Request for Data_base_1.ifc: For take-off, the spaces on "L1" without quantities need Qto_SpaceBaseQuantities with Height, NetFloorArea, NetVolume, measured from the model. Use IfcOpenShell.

First a look at what the model holds.

```python
import ifcopenshell
import ifcopenshell.util.element
import ifcopenshell.util.unit

model = ifcopenshell.open("Data_base_1.ifc")
print(model.schema)
for unit_type in ("LENGTHUNIT", "AREAUNIT", "VOLUMEUNIT"):
    print(unit_type, ifcopenshell.util.unit.calculate_unit_scale(model, unit_type))
storey = next(s for s in model.by_type("IfcBuildingStorey") if s.Name == "L1")
spaces = [e for e in ifcopenshell.util.element.get_decomposition(storey) if e.is_a("IfcSpace")]
for e in sorted(spaces, key=lambda e: e.id()):
    print(e.id(), e.is_a(), e.Name, list(ifcopenshell.util.element.get_psets(e, qtos_only=True)), sep=" | ")
```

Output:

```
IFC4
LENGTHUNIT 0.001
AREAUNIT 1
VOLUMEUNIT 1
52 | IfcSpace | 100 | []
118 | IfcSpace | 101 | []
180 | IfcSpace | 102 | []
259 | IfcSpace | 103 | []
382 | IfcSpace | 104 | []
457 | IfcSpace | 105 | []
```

```python
import ifcopenshell
import ifcopenshell.api.pset
import ifcopenshell.geom
import ifcopenshell.util.element
import ifcopenshell.util.shape
import ifcopenshell.util.unit

model = ifcopenshell.open("Data_base_1.ifc")
unit_scale = ifcopenshell.util.unit.calculate_unit_scale(model)
area_scale = ifcopenshell.util.unit.calculate_unit_scale(model, "AREAUNIT")
volume_scale = ifcopenshell.util.unit.calculate_unit_scale(model, "VOLUMEUNIT")
settings = ifcopenshell.geom.settings()

storey = next(s for s in model.by_type("IfcBuildingStorey") if s.Name == "L1")
spaces = [e for e in ifcopenshell.util.element.get_decomposition(storey) if e.is_a("IfcSpace")]

for e in sorted(spaces, key=lambda e: e.id()):
    if ifcopenshell.util.element.get_psets(e, qtos_only=True, should_inherit=False):
        continue
    # Geometry comes back in metres, in the element's own axes.
    shape = ifcopenshell.geom.create_shape(settings, e)
    values = {
        "Height": ifcopenshell.util.shape.get_z(shape.geometry) / unit_scale,
        "NetFloorArea": ifcopenshell.util.shape.get_footprint_area(shape.geometry) / area_scale,
        "NetVolume": ifcopenshell.util.shape.get_volume(shape.geometry) / volume_scale,
    }
    qto = ifcopenshell.api.pset.add_qto(model, product=e, name="Qto_SpaceBaseQuantities")
    ifcopenshell.api.pset.edit_qto(model, qto=qto, properties=values)
    print(e.id(), {k: round(v, 3) for k, v in values.items()})

model.write("Data_base_1_updated.ifc")
```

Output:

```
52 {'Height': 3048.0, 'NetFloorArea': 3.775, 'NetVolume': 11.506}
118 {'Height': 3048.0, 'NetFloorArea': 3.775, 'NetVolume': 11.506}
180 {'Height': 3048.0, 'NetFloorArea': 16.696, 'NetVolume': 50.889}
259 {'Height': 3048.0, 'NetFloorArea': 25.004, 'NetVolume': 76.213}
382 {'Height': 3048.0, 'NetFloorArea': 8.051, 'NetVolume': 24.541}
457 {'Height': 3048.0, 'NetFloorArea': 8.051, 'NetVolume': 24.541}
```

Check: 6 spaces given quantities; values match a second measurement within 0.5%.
